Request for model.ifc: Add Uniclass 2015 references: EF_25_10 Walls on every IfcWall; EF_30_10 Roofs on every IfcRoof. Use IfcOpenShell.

First a look at what the model holds.

```python
import ifcopenshell

model = ifcopenshell.open("model.ifc")
print(model.schema)
print("classifications:", [c.Name for c in model.by_type("IfcClassification")])
for ifc_class in ("IfcDoor", "IfcRoof", "IfcStair", "IfcWall", "IfcWindow"):
    print(ifc_class, len(model.by_type(ifc_class)))
```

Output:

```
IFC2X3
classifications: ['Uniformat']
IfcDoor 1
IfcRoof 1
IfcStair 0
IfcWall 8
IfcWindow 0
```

```python
import ifcopenshell
import ifcopenshell.api.classification

model = ifcopenshell.open("model.ifc")

# IFC2X3 requires Source and Edition and has no link from the project to the system.
system = model.create_entity("IfcClassification", Source="NBS", Edition="2015", Name="Uniclass 2015")

codes = {
    "IfcWall": ("EF_25_10", "Walls"),
    "IfcRoof": ("EF_30_10", "Roofs"),
}
for ifc_class, (code, name) in codes.items():
    products = model.by_type(ifc_class)
    ifcopenshell.api.classification.add_reference(
        model, products=products, classification=system, identification=code, name=name
    )
    print(code, len(products))

model.write("model_updated.ifc")
```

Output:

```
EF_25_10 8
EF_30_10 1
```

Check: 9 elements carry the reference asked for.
